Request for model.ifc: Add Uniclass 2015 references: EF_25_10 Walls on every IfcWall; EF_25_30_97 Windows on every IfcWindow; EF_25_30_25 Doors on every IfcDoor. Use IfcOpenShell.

First a look at what the model holds.

```python
import ifcopenshell

model = ifcopenshell.open("model.ifc")
print(model.schema)
print("classifications:", [c.Name for c in model.by_type("IfcClassification")])
for ifc_class in ("IfcDoor", "IfcRoof", "IfcStair", "IfcWall", "IfcWindow"):
    print(ifc_class, len(model.by_type(ifc_class)))
```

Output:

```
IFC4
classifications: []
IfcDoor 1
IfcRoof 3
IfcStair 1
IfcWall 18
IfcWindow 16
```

```python
import ifcopenshell
import ifcopenshell.api.classification

model = ifcopenshell.open("model.ifc")

system = ifcopenshell.api.classification.add_classification(model, classification="Uniclass 2015")

codes = {
    "IfcWall": ("EF_25_10", "Walls"),
    "IfcWindow": ("EF_25_30_97", "Windows"),
    "IfcDoor": ("EF_25_30_25", "Doors"),
}
for ifc_class, (code, name) in codes.items():
    products = model.by_type(ifc_class)
    ifcopenshell.api.classification.add_reference(
        model, products=products, classification=system, identification=code, name=name
    )
    print(code, len(products))

model.write("model_updated.ifc")
```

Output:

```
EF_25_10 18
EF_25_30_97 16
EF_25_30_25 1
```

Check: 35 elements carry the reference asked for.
